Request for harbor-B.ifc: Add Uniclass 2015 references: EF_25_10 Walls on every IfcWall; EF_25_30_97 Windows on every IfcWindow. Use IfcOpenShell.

First a look at what the model holds.

```python
import ifcopenshell

model = ifcopenshell.open("harbor-B.ifc")
print(model.schema)
print("classifications:", [c.Name for c in model.by_type("IfcClassification")])
for ifc_class in ("IfcDoor", "IfcRoof", "IfcStair", "IfcWall", "IfcWindow"):
    print(ifc_class, len(model.by_type(ifc_class)))
```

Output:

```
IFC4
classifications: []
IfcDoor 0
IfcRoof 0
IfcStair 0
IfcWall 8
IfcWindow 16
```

```python
import ifcopenshell
import ifcopenshell.api.classification

model = ifcopenshell.open("harbor-B.ifc")

system = ifcopenshell.api.classification.add_classification(model, classification="Uniclass 2015")

codes = {
    "IfcWall": ("EF_25_10", "Walls"),
    "IfcWindow": ("EF_25_30_97", "Windows"),
}
for ifc_class, (code, name) in codes.items():
    products = model.by_type(ifc_class)
    ifcopenshell.api.classification.add_reference(
        model, products=products, classification=system, identification=code, name=name
    )
    print(code, len(products))

model.write("harbor-B-out.ifc")
```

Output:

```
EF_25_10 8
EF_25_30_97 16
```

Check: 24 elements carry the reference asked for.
